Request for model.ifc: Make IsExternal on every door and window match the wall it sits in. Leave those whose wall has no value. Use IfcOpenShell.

First a look at what the model holds.

```python
import ifcopenshell
import ifcopenshell.util.element

model = ifcopenshell.open("model.ifc")
print(model.schema)
seen = {}
for e in model.by_type("IfcDoor") + model.by_type("IfcWindow"):
    if not e.FillsVoids:
        continue
    host = e.FillsVoids[0].RelatingOpeningElement.VoidsElements[0].RelatingBuildingElement
    own = ifcopenshell.util.element.get_pset(e, f"Pset_{e.is_a()[3:].removesuffix('StandardCase')}Common", "IsExternal")
    wall = ifcopenshell.util.element.get_pset(host, "Pset_WallCommon", "IsExternal")
    seen[e.is_a(), own, wall] = seen.get((e.is_a(), own, wall), 0) + 1
for (cls, own, wall), count in sorted(seen.items(), key=str):
    print(count, cls, "IsExternal:", own, "| host wall:", wall)
```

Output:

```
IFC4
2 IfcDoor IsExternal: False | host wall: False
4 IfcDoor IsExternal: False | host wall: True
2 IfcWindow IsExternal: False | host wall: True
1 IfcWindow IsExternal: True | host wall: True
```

```python
import ifcopenshell
import ifcopenshell.api.pset
import ifcopenshell.util.element

model = ifcopenshell.open("model.ifc")

count = 0
for ifc_class, pset_name in (("IfcDoor", "Pset_DoorCommon"), ("IfcWindow", "Pset_WindowCommon")):
    for e in model.by_type(ifc_class):
        if not e.FillsVoids:
            continue
        host = e.FillsVoids[0].RelatingOpeningElement.VoidsElements[0].RelatingBuildingElement
        external = ifcopenshell.util.element.get_pset(host, "Pset_WallCommon", "IsExternal")
        if external is None or ifcopenshell.util.element.get_pset(e, pset_name, "IsExternal") == external:
            continue
        pset = ifcopenshell.api.pset.add_pset(model, product=e, name=pset_name)
        ifcopenshell.api.pset.edit_pset(model, pset=pset, properties={"IsExternal": external})
        count += 1

print(count, "updated")

model.write("model_edited.ifc")
```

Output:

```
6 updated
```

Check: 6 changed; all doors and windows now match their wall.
